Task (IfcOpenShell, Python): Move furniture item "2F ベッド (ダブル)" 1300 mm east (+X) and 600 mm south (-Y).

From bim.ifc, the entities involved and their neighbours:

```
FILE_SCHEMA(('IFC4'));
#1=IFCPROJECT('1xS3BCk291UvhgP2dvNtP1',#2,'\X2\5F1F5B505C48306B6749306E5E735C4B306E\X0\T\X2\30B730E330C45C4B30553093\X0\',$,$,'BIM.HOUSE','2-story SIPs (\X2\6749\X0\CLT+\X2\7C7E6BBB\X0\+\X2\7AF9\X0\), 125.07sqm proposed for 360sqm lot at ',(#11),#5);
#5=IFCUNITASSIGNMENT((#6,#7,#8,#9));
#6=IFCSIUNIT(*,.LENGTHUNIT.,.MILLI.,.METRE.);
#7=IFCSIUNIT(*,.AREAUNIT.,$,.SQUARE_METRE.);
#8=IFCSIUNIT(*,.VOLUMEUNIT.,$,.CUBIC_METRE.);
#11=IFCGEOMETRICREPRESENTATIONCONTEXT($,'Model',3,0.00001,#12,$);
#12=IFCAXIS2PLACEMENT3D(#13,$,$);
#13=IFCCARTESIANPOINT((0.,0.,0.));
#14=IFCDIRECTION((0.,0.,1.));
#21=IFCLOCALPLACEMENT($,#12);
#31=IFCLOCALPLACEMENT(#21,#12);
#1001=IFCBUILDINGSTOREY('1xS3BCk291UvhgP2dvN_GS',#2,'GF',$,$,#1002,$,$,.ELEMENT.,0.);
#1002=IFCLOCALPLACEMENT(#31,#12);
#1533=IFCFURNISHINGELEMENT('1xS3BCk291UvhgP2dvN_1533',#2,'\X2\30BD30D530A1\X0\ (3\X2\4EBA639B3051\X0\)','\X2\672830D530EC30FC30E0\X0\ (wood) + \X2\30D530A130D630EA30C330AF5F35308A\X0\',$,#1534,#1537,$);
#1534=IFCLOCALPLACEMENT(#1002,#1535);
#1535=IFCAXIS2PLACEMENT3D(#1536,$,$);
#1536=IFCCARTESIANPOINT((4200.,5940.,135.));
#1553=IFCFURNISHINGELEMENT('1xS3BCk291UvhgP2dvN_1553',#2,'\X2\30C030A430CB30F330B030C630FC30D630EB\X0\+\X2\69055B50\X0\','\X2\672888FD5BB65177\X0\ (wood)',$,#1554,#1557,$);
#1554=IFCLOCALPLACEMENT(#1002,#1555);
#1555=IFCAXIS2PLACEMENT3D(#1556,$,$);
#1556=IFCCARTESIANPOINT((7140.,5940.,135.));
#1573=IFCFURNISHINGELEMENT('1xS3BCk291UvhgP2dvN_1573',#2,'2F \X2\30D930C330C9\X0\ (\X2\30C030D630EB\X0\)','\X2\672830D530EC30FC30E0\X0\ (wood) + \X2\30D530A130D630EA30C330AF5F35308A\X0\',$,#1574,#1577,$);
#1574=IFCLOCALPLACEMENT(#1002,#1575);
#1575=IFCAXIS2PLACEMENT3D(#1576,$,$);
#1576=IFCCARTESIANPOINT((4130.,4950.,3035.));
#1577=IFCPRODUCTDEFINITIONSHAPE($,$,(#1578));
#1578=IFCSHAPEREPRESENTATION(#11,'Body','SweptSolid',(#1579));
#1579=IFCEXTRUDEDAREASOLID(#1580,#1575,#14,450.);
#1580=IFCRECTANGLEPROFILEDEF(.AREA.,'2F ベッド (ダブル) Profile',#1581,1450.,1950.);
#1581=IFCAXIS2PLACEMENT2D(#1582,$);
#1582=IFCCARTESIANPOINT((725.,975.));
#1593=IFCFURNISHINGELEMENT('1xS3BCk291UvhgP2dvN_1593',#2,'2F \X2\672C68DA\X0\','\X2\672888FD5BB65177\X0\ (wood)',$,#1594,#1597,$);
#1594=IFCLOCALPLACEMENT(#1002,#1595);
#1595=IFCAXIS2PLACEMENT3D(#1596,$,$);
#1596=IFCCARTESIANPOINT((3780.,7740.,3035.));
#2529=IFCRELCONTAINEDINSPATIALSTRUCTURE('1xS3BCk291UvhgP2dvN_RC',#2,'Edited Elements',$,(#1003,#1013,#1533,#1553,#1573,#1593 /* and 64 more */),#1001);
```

```python
import ifcopenshell
import ifcopenshell.api.geometry
import ifcopenshell.util.placement
import ifcopenshell.util.unit

model = ifcopenshell.open("bim.ifc")
unit_scale = ifcopenshell.util.unit.calculate_unit_scale(model)

item = model.by_guid("1xS3BCk291UvhgP2dvN_1573")
matrix = ifcopenshell.util.placement.get_local_placement(item.ObjectPlacement)
matrix[0, 3] += 1.3 / unit_scale
matrix[1, 3] -= 0.6 / unit_scale
ifcopenshell.api.geometry.edit_object_placement(model, product=item, matrix=matrix, is_si=False)

print(ifcopenshell.util.placement.get_local_placement(item.ObjectPlacement).round(3) + 0.0)

model.write("bim_v2.ifc")
```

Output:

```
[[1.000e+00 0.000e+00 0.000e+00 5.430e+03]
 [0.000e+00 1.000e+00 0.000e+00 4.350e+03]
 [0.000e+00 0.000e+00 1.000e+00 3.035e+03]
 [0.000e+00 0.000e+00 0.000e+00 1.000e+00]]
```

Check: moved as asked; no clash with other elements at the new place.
